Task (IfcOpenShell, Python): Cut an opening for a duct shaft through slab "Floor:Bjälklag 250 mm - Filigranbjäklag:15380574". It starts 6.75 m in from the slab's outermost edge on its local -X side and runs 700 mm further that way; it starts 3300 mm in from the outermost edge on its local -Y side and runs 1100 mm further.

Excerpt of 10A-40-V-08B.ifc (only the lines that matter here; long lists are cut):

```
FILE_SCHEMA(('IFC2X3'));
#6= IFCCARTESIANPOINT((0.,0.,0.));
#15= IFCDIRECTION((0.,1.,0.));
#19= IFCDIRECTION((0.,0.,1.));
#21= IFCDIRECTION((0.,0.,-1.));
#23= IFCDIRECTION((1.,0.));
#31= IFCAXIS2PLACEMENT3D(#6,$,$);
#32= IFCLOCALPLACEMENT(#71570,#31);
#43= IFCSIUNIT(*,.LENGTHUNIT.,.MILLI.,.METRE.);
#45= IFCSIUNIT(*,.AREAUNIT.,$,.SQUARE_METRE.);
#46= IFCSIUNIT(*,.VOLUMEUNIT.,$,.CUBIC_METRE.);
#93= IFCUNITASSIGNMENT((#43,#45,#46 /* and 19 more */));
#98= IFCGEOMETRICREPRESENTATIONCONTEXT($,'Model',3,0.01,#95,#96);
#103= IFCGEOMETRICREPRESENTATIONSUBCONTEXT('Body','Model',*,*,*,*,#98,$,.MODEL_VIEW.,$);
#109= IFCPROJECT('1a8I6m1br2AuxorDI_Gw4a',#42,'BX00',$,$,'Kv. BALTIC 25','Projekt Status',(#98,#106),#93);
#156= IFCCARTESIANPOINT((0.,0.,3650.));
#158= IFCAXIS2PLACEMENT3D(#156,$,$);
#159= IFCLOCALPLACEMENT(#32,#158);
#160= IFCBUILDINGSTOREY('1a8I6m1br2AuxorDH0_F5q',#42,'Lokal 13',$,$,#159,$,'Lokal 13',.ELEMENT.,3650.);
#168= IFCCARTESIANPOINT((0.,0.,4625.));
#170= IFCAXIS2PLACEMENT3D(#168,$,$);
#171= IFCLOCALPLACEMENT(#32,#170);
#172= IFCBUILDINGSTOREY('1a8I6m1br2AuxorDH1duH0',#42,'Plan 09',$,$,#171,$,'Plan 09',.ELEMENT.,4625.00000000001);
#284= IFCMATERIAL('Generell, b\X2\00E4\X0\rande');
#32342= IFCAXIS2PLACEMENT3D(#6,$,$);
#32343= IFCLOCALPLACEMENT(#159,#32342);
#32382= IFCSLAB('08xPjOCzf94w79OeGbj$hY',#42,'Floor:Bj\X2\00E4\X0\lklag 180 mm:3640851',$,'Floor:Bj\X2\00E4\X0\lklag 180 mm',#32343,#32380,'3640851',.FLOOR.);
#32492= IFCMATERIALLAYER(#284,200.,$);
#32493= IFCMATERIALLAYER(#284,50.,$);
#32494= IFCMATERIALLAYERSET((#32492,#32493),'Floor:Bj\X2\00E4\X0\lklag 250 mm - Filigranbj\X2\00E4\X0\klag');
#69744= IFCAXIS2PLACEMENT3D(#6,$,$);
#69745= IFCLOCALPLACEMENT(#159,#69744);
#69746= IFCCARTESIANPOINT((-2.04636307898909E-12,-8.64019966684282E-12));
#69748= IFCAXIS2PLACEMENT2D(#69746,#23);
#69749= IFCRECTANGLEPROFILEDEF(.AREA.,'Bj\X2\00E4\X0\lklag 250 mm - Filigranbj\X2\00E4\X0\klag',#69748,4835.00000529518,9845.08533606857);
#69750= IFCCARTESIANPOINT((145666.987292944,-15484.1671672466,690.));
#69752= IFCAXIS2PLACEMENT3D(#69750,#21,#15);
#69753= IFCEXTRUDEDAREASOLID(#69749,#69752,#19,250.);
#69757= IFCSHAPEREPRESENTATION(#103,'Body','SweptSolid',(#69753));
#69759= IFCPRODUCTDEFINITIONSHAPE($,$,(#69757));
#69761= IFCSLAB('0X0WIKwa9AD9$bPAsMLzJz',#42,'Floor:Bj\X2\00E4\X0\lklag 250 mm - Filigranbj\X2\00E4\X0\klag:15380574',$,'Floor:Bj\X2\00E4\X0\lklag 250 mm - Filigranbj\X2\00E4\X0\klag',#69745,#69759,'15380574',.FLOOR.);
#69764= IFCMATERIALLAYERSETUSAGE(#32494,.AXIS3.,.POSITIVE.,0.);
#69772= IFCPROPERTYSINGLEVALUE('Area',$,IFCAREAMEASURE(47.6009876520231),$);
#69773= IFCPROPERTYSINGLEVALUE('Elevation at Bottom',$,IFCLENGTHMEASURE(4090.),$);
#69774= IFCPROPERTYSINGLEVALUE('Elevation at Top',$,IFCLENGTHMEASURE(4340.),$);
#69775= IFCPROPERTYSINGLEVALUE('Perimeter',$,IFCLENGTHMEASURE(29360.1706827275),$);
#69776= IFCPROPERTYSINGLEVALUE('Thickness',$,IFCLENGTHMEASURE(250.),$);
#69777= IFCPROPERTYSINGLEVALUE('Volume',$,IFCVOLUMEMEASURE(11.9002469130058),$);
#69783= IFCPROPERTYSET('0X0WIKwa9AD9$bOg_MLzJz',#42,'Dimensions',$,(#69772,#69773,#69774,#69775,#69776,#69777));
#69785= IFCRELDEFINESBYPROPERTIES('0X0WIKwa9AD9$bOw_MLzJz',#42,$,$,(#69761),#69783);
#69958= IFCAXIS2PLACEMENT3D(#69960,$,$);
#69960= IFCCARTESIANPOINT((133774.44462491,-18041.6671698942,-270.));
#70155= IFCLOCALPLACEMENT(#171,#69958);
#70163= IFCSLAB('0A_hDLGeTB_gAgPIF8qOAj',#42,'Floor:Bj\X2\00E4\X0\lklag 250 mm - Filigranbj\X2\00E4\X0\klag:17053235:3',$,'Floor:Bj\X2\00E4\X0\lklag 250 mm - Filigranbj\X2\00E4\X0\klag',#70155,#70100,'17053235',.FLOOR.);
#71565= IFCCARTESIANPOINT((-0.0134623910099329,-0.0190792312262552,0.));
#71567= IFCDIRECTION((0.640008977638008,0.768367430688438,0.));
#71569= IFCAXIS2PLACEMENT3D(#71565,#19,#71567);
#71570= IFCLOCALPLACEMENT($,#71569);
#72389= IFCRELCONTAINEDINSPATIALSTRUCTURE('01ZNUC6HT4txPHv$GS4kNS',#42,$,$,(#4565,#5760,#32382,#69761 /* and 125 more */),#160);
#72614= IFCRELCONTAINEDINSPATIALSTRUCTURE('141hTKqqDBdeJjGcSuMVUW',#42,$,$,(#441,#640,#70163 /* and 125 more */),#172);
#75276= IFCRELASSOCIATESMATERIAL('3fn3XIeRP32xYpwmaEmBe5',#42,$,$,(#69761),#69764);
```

```python
import numpy as np
import ifcopenshell
import ifcopenshell.api.feature
import ifcopenshell.api.geometry
import ifcopenshell.api.pset
import ifcopenshell.api.root
import ifcopenshell.geom
import ifcopenshell.util.element
import ifcopenshell.util.placement
import ifcopenshell.util.representation
import ifcopenshell.util.shape
import ifcopenshell.util.unit

model = ifcopenshell.open("10A-40-V-08B.ifc")
unit_scale = ifcopenshell.util.unit.calculate_unit_scale(model)
area_scale = ifcopenshell.util.unit.calculate_unit_scale(model, "AREAUNIT")
volume_scale = ifcopenshell.util.unit.calculate_unit_scale(model, "VOLUMEUNIT")
settings = ifcopenshell.geom.settings()


def volume(element):
    """Net volume in cubic metres, openings subtracted."""
    shape = ifcopenshell.geom.create_shape(settings, element)
    return ifcopenshell.util.shape.get_volume(shape.geometry)


slab = model.by_guid("0X0WIKwa9AD9$bPAsMLzJz")
before = volume(slab)

# Extent in the slab's own axes, in metres. The edges named are its -X and -Y sides.
slab_shape = ifcopenshell.geom.create_shape(settings, slab)
vertices = ifcopenshell.util.shape.get_vertices(slab_shape.geometry)
x_min, y_min, bottom = vertices.min(axis=0)
top = vertices[:, 2].max()

opening = ifcopenshell.api.root.create_entity(model, ifc_class="IfcOpeningElement", name="Duct shaft opening")
context = ifcopenshell.util.representation.get_context(model, "Model", "Body", "MODEL_VIEW")
width, depth = 0.7, 1.1
outline = [(0.0, 0.0), (width, 0.0), (width, depth), (0.0, depth), (0.0, 0.0)]
# Overshoot both faces by 50 mm so the cut is clean.
shape = ifcopenshell.api.geometry.add_slab_representation(
    model, context=context, depth=top - bottom + 0.1, polyline=outline
)
ifcopenshell.api.geometry.assign_representation(model, product=opening, representation=shape)

matrix = ifcopenshell.util.placement.get_local_placement(slab.ObjectPlacement)
matrix[:, 3] = matrix @ np.append(np.array([x_min + 6.75, y_min + 3.3, bottom - 0.05]) / unit_scale, 1.0)
ifcopenshell.api.geometry.edit_object_placement(model, product=opening, matrix=matrix, is_si=False)
ifcopenshell.api.feature.add_feature(model, feature=opening, element=slab)

after = volume(slab)

# Update the slab's stored quantities.
pset = model.by_id(ifcopenshell.util.element.get_pset(slab, "Dimensions", should_inherit=False)["id"])
ifcopenshell.api.pset.edit_pset(model, pset=pset, properties={
    "Area": model.create_entity("IfcAreaMeasure", after / (top - bottom) / area_scale),
    "Volume": model.create_entity("IfcVolumeMeasure", after / volume_scale),
})

print(f"slab volume {before:.3f} -> {after:.3f} m3")

model.write("10A-40-V-08B_v2.ifc")
```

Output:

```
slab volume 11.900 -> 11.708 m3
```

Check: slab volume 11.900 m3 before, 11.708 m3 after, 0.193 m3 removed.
